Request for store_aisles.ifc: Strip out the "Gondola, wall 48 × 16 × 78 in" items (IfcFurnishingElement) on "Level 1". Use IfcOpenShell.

First a look at what the model holds.

```python
import ifcopenshell
import ifcopenshell.util.element

model = ifcopenshell.open("store_aisles.ifc")
print(model.schema)
storey = next(s for s in model.by_type("IfcBuildingStorey") if s.Name == "Level 1")
furniture = [e for e in ifcopenshell.util.element.get_decomposition(storey) if e.is_a("IfcFurnishingElement")]
seen = {}
for e in furniture:
    element_type = ifcopenshell.util.element.get_type(e)
    name = element_type.Name if element_type not in (None, e) else None
    seen[name] = seen.get(name, 0) + 1
for name, count in sorted(seen.items(), key=str):
    print(count, "x", name)
```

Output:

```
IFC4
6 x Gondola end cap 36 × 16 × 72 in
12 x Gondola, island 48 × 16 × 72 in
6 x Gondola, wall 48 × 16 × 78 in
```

```python
import ifcopenshell
import ifcopenshell.api.root
import ifcopenshell.util.element

model = ifcopenshell.open("store_aisles.ifc")

storey = next(s for s in model.by_type("IfcBuildingStorey") if s.Name == "Level 1")
furniture = [e for e in ifcopenshell.util.element.get_decomposition(storey) if e.is_a("IfcFurnishingElement")]
targets = [e for e in furniture if (t := ifcopenshell.util.element.get_type(e)) not in (None, e) and t.Name == "Gondola, wall 48 × 16 × 78 in"]

for e in targets:
    ifcopenshell.api.root.remove_product(model, product=e)
print(len(targets), "removed")

model.write("store_aisles_v2.ifc")
```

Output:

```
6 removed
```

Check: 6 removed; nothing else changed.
